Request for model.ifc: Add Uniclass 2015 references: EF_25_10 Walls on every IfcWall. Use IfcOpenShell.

First a look at what the model holds.

```python
import ifcopenshell

model = ifcopenshell.open("model.ifc")
print(model.schema)
print("classifications:", [c.Name for c in model.by_type("IfcClassification")])
for ifc_class in ("IfcDoor", "IfcRoof", "IfcStair", "IfcWall", "IfcWindow"):
    print(ifc_class, len(model.by_type(ifc_class)))
```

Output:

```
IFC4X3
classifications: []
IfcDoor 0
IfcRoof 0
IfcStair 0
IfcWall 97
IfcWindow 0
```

```python
import ifcopenshell
import ifcopenshell.api.classification

model = ifcopenshell.open("model.ifc")

system = ifcopenshell.api.classification.add_classification(model, classification="Uniclass 2015")

codes = {
    "IfcWall": ("EF_25_10", "Walls"),
}
for ifc_class, (code, name) in codes.items():
    products = model.by_type(ifc_class)
    ifcopenshell.api.classification.add_reference(
        model, products=products, classification=system, identification=code, name=name
    )
    print(code, len(products))

model.write("model_rev.ifc")
```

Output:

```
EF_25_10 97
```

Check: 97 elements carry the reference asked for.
